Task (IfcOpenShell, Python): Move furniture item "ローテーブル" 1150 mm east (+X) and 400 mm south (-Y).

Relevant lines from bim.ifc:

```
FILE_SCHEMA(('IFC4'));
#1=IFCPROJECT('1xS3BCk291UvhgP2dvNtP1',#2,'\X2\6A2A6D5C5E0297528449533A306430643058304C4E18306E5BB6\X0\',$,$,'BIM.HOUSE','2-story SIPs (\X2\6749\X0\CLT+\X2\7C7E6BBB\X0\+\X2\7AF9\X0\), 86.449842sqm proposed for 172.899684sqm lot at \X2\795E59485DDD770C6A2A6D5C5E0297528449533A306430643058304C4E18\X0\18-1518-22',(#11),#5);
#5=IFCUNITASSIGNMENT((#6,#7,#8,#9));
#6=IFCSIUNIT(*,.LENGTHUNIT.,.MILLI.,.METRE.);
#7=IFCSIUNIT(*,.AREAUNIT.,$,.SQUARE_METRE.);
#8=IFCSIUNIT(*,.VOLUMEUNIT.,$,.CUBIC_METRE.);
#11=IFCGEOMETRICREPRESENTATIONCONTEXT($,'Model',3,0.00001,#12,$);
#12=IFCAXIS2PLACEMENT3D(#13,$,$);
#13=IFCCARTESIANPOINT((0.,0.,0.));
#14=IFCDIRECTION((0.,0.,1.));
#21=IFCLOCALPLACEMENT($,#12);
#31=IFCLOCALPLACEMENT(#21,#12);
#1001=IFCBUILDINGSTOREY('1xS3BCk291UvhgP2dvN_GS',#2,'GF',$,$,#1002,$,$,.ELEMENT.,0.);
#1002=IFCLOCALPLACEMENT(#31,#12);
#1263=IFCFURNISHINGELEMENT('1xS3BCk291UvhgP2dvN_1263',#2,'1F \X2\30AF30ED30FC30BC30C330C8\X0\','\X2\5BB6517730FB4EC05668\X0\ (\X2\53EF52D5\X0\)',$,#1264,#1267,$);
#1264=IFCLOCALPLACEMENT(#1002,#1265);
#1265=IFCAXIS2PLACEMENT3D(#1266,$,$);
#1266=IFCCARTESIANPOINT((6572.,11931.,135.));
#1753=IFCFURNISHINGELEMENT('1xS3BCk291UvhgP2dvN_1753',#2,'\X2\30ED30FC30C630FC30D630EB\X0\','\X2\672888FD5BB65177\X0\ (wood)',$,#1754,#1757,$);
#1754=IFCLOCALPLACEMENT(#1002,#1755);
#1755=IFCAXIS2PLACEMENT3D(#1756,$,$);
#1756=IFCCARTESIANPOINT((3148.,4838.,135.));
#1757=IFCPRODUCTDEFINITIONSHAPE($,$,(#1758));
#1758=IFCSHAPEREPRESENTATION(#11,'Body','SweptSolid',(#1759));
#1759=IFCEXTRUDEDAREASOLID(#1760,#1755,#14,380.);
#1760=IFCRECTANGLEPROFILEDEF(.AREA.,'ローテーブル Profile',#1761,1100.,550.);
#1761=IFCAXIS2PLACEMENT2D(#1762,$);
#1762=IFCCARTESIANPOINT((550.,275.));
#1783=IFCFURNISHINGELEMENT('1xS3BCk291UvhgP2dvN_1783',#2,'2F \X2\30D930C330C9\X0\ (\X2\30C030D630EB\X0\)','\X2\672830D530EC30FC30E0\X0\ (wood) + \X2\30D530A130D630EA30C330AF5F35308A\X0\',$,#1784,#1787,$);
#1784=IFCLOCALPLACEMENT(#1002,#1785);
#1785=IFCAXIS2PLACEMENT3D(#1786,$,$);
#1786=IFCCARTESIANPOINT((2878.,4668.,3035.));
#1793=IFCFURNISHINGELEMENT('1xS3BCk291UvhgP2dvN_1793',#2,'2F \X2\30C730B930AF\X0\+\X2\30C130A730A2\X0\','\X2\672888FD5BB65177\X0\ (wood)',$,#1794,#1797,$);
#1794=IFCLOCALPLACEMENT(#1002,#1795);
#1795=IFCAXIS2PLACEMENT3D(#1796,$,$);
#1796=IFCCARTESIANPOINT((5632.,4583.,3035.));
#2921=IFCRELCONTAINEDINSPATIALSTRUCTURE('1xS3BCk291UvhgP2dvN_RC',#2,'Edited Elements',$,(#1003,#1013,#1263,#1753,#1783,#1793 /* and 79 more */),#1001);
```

```python
import ifcopenshell
import ifcopenshell.api.geometry
import ifcopenshell.util.placement
import ifcopenshell.util.unit

model = ifcopenshell.open("bim.ifc")
unit_scale = ifcopenshell.util.unit.calculate_unit_scale(model)

item = model.by_id(1753)
matrix = ifcopenshell.util.placement.get_local_placement(item.ObjectPlacement)
matrix[0, 3] += 1.15 / unit_scale
matrix[1, 3] -= 0.4 / unit_scale
ifcopenshell.api.geometry.edit_object_placement(model, product=item, matrix=matrix, is_si=False)

print(ifcopenshell.util.placement.get_local_placement(item.ObjectPlacement).round(3) + 0.0)

model.write("bim_edited.ifc")
```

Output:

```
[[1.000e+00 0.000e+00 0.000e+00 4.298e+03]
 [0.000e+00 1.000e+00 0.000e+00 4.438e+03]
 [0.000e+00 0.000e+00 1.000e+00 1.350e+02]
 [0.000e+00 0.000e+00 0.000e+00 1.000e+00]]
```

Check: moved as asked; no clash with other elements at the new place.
